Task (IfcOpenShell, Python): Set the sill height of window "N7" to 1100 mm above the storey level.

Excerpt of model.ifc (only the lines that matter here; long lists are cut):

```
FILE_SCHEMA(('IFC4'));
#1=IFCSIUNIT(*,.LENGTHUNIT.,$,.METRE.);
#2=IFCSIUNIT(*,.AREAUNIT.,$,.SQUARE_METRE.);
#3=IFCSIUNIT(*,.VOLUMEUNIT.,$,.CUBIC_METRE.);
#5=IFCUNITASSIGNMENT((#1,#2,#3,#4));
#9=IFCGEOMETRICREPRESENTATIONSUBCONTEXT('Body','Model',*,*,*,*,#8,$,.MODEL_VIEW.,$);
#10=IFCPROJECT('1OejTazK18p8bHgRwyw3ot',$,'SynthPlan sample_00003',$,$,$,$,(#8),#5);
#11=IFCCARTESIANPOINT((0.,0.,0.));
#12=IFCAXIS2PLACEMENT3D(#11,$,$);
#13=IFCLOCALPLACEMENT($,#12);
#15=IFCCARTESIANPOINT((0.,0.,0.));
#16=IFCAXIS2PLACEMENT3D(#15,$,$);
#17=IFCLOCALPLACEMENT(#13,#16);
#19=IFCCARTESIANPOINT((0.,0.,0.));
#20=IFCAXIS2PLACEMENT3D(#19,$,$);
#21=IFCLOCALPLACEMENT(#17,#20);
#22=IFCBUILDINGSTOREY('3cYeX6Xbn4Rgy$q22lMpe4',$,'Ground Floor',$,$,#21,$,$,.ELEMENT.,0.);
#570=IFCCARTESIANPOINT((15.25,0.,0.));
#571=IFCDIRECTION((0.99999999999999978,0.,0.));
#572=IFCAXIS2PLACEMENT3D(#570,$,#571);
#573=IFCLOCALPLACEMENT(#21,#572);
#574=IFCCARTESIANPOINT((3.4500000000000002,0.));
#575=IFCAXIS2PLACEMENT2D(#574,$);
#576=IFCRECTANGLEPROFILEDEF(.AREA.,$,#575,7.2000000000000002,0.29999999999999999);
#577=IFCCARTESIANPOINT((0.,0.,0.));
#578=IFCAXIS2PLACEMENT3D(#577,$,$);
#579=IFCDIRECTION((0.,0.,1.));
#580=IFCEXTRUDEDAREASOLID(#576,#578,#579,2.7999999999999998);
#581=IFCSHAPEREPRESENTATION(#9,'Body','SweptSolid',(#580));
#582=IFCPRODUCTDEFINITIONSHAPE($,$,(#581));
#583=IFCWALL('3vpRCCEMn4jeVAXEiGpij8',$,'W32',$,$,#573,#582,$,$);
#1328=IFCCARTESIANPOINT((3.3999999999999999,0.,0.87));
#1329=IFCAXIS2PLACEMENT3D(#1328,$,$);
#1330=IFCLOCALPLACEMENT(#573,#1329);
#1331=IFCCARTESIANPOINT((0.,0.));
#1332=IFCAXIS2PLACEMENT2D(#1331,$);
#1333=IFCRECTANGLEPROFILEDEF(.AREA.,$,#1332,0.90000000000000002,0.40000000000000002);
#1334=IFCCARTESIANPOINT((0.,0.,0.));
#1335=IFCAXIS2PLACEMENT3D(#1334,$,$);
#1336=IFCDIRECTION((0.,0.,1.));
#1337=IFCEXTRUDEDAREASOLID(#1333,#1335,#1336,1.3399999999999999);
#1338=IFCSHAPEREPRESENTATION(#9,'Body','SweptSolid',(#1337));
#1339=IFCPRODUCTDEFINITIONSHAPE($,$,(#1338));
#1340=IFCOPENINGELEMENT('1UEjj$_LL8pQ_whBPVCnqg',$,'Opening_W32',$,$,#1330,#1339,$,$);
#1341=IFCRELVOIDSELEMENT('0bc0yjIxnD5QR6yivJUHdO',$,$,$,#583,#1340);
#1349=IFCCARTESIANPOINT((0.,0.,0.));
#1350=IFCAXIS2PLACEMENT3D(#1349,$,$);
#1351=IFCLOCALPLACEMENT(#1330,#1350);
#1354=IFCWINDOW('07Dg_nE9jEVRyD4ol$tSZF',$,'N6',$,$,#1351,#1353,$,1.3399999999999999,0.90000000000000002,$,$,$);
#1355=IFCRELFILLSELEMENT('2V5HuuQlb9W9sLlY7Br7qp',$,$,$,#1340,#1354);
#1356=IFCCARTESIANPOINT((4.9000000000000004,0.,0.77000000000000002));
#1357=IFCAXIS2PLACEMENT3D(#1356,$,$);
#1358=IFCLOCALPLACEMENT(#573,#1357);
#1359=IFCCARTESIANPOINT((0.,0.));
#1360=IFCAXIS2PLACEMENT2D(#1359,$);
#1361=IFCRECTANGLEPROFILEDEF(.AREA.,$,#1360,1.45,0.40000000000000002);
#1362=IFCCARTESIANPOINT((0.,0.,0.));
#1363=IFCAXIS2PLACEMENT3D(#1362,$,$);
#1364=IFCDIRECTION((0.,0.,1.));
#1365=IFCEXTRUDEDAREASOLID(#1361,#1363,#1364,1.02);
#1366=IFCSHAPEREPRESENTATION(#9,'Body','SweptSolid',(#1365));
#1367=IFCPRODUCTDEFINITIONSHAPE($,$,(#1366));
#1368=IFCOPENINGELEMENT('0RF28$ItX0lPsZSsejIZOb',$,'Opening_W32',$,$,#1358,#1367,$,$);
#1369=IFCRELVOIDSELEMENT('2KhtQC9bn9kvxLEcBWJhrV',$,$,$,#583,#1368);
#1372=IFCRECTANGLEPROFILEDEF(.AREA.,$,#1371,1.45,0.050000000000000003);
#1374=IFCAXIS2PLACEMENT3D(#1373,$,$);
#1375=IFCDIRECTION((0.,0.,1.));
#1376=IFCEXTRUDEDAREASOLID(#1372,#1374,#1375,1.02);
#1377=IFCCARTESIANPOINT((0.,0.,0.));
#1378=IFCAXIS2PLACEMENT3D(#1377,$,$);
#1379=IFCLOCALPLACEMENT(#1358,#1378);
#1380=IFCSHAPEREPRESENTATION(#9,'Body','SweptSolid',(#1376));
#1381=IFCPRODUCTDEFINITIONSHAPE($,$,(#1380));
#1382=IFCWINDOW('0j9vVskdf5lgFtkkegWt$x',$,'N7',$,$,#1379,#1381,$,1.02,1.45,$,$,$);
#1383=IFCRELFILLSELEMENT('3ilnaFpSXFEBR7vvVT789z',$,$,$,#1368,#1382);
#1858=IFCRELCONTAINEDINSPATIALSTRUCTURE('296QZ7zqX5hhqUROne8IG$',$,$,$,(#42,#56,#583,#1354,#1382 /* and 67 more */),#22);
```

```python
import numpy as np
import ifcopenshell
import ifcopenshell.api.geometry
import ifcopenshell.geom
import ifcopenshell.util.element
import ifcopenshell.util.placement
import ifcopenshell.util.shape
import ifcopenshell.util.unit

model = ifcopenshell.open("model.ifc")
unit_scale = ifcopenshell.util.unit.calculate_unit_scale(model)

window = model.by_id(1382)
opening = window.FillsVoids[0].RelatingOpeningElement
storey = ifcopenshell.util.element.get_container(window, ifc_class="IfcBuildingStorey")
level = ifcopenshell.util.placement.get_local_placement(storey.ObjectPlacement)[2, 3]

# The opening's origin need not be at the sill, so measure its lowest point.
shape = ifcopenshell.geom.create_shape(ifcopenshell.geom.settings(), opening)
bottom = ifcopenshell.util.shape.get_shape_bottom_elevation(shape, shape.geometry) / unit_scale
dz = level + 1.1 - bottom

shift = np.array([0.0, 0.0, dz])
# The window is placed relative to its opening, so it follows when the opening moves.
matrix = ifcopenshell.util.placement.get_local_placement(opening.ObjectPlacement)
matrix[:3, 3] += shift
ifcopenshell.api.geometry.edit_object_placement(
    model, product=opening, matrix=matrix, is_si=False, should_transform_children=True
)

print(f"moved by {dz * unit_scale:+.3f} m")

model.write("model_updated.ifc")
```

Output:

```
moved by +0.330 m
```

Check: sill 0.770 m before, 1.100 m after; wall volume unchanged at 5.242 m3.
